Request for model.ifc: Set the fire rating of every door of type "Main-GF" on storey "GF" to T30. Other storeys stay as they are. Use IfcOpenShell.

First a look at what the model holds.

```python
import ifcopenshell
import ifcopenshell.util.element

model = ifcopenshell.open("model.ifc")
print(model.schema)
storey = next(s for s in model.by_type("IfcBuildingStorey") if s.Name == "GF")
doors = [e for e in ifcopenshell.util.element.get_decomposition(storey) if e.is_a("IfcDoor")]
seen = {}
for e in doors:
    element_type = ifcopenshell.util.element.get_type(e)
    key = (element_type.Name if element_type != e and element_type else None, ifcopenshell.util.element.get_pset(e, "Pset_DoorCommon", "FireRating"))
    seen[key] = seen.get(key, 0) + 1
for (name, value), count in sorted(seen.items(), key=str):
    print(count, "x", name, "|", value)
```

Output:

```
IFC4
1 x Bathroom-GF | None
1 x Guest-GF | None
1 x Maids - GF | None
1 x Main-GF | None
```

```python
import ifcopenshell
import ifcopenshell.api.pset
import ifcopenshell.util.element

model = ifcopenshell.open("model.ifc")

storey = next(s for s in model.by_type("IfcBuildingStorey") if s.Name == "GF")
doors = [e for e in ifcopenshell.util.element.get_decomposition(storey) if e.is_a("IfcDoor")]

count = 0
for e in doors:
    element_type = ifcopenshell.util.element.get_type(e)
    if element_type in (None, e) or element_type.Name != "Main-GF":
        continue
    # add_pset returns the element's existing set when there is one.
    pset = ifcopenshell.api.pset.add_pset(model, product=e, name="Pset_DoorCommon")
    ifcopenshell.api.pset.edit_pset(model, pset=pset, properties={"FireRating": "T30"})
    count += 1

print(count, "doors updated")

model.write("model_edited.ifc")
```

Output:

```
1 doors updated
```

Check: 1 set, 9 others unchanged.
